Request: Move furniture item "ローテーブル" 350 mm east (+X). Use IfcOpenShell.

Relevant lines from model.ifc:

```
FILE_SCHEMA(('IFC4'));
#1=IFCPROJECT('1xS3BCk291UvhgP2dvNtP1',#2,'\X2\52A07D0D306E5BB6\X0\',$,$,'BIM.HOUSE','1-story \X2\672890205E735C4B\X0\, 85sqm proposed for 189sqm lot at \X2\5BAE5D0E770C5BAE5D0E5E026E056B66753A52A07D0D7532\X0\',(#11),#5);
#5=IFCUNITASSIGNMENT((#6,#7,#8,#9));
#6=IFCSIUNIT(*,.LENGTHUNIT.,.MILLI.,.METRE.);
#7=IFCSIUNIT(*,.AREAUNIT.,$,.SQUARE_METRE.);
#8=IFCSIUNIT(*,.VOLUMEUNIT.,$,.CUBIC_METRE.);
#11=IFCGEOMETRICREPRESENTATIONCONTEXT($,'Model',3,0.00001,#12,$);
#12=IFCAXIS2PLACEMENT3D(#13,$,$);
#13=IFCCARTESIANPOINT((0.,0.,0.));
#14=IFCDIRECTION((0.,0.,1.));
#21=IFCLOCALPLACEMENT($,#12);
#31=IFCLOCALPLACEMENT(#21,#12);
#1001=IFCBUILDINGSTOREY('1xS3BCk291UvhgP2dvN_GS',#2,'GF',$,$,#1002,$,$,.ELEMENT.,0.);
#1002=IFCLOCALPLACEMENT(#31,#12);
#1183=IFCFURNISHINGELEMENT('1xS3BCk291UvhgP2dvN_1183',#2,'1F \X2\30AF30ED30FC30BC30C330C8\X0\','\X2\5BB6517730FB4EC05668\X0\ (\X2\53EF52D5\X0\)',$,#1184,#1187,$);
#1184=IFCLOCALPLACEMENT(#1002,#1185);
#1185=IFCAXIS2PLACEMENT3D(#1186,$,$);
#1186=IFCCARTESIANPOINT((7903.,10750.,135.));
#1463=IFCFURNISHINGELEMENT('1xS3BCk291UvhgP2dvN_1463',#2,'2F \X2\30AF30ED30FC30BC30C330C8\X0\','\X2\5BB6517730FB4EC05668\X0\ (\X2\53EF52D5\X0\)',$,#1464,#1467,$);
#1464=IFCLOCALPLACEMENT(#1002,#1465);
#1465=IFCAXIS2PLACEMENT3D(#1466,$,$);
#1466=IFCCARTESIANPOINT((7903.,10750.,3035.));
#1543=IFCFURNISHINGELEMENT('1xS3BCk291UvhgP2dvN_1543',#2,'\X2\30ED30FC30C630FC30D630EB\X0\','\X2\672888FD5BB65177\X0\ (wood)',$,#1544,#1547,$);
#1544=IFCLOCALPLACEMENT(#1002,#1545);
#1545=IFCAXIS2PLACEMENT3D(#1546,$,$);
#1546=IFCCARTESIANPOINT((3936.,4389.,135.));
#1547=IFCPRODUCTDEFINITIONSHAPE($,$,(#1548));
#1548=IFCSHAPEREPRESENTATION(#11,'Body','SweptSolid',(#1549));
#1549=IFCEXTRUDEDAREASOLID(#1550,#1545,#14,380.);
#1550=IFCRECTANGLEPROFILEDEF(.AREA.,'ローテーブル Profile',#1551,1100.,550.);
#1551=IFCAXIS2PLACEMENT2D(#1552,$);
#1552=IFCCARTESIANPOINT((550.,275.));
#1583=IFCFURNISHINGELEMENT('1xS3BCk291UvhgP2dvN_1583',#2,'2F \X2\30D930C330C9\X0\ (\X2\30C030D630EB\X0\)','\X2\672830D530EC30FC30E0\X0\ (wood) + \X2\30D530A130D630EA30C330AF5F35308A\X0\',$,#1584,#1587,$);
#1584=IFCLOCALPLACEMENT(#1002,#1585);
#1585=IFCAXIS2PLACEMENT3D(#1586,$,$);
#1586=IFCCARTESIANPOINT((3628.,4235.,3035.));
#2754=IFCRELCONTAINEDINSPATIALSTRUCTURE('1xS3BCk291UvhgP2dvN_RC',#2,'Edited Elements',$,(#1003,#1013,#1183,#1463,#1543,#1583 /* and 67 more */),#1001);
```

```python
import ifcopenshell
import ifcopenshell.api.geometry
import ifcopenshell.util.placement
import ifcopenshell.util.unit

model = ifcopenshell.open("model.ifc")
unit_scale = ifcopenshell.util.unit.calculate_unit_scale(model)

item = model.by_guid("1xS3BCk291UvhgP2dvN_1543")
matrix = ifcopenshell.util.placement.get_local_placement(item.ObjectPlacement)
matrix[0, 3] += 0.35 / unit_scale
ifcopenshell.api.geometry.edit_object_placement(model, product=item, matrix=matrix, is_si=False)

print(ifcopenshell.util.placement.get_local_placement(item.ObjectPlacement).round(3) + 0.0)

model.write("model-out.ifc")
```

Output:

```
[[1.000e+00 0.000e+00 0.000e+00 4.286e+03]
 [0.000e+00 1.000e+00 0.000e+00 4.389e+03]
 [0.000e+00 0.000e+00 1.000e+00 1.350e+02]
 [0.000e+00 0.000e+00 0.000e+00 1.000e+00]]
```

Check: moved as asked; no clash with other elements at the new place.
